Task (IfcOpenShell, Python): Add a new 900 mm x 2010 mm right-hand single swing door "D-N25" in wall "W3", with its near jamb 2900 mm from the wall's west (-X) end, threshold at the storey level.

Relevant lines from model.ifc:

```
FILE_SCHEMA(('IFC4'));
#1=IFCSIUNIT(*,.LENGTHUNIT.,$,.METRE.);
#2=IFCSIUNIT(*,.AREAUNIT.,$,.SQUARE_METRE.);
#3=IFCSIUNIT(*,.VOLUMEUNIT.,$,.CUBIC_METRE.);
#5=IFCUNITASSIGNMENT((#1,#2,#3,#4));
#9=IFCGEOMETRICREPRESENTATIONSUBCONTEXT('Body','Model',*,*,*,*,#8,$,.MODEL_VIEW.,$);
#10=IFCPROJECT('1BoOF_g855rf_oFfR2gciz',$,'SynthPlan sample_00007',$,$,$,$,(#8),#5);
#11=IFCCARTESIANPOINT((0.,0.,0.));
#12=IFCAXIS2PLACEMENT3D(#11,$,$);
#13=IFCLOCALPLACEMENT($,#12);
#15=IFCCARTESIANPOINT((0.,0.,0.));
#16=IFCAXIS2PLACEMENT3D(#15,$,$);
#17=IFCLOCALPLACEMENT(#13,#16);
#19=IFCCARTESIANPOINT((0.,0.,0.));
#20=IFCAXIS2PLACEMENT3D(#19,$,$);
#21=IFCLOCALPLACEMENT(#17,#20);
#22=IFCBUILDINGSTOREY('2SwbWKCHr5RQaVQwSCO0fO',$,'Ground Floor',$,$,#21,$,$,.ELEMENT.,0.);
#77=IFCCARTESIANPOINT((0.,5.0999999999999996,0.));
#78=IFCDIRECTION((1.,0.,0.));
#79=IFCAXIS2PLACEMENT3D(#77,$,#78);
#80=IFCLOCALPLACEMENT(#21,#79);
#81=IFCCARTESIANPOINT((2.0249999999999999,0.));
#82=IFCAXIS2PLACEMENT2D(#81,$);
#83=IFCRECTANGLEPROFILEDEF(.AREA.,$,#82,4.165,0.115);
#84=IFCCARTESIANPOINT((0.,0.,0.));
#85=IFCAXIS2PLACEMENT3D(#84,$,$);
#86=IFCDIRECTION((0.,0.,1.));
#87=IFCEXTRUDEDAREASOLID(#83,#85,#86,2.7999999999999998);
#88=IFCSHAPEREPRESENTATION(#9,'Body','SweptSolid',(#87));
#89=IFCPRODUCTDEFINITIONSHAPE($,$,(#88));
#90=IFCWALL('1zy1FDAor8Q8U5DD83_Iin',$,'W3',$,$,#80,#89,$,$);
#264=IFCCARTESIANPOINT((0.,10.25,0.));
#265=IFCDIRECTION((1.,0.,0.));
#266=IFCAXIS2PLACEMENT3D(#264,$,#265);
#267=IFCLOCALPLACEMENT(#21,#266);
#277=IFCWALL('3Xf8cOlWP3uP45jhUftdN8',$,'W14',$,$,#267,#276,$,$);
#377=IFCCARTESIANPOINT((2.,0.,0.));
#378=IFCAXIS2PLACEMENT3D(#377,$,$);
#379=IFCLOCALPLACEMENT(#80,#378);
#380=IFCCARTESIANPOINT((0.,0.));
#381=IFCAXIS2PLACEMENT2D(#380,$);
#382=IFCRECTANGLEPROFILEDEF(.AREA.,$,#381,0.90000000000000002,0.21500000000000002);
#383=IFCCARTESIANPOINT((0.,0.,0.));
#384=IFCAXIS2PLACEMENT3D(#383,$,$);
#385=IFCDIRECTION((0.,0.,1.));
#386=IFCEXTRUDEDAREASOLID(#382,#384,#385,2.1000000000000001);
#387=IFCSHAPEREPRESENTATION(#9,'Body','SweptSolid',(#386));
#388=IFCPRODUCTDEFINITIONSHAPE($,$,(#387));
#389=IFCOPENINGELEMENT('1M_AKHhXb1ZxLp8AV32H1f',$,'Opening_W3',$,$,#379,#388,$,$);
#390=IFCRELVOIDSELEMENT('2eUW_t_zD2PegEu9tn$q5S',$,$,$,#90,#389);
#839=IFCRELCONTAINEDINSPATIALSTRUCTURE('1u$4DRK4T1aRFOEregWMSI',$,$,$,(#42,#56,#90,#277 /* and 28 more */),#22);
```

```python
import numpy as np
import ifcopenshell
import ifcopenshell.api.feature
import ifcopenshell.api.geometry
import ifcopenshell.api.root
import ifcopenshell.api.spatial
import ifcopenshell.geom
import ifcopenshell.util.element
import ifcopenshell.util.placement
import ifcopenshell.util.representation
import ifcopenshell.util.shape
import ifcopenshell.util.unit

model = ifcopenshell.open("model.ifc")
unit_scale = ifcopenshell.util.unit.calculate_unit_scale(model)
settings = ifcopenshell.geom.settings()


def volume(element):
    """Net volume in cubic metres, openings subtracted."""
    shape = ifcopenshell.geom.create_shape(settings, element)
    return ifcopenshell.util.shape.get_volume(shape.geometry)


wall = model.by_guid("1zy1FDAor8Q8U5DD83_Iin")
storey = ifcopenshell.util.element.get_container(wall, ifc_class="IfcBuildingStorey")
context = ifcopenshell.util.representation.get_context(model, "Model", "Body", "MODEL_VIEW")
before = volume(wall)

width, height, from_end, sill = 0.9, 2.01, 2.9, 0.0  # metres

# The wall runs along its own X axis, and the end named is its -X end.
wall_shape = ifcopenshell.geom.create_shape(settings, wall)
x, y, z = ifcopenshell.util.shape.get_vertices(wall_shape.geometry).T
start = x.min() + from_end
face, thickness = float(y.min()), float(y.max() - y.min())
wall_matrix = ifcopenshell.util.placement.get_local_placement(wall.ObjectPlacement)
level = ifcopenshell.util.placement.get_local_placement(storey.ObjectPlacement)[2, 3]


def in_wall(x, y):
    """Placement at x, y metres in the wall's axes, at sill height."""
    matrix = wall_matrix.copy()
    matrix[:, 3] = wall_matrix @ np.array([x / unit_scale, y / unit_scale, 0.0, 1.0])
    matrix[2, 3] = level + sill / unit_scale
    return matrix


# Opening: a box that overshoots both wall faces by 50 mm.
opening = ifcopenshell.api.root.create_entity(model, ifc_class="IfcOpeningElement", predefined_type="OPENING")
box = ifcopenshell.api.geometry.add_wall_representation(
    model, context=context, length=width, height=height, thickness=thickness + 0.1
)
ifcopenshell.api.geometry.assign_representation(model, product=opening, representation=box)
ifcopenshell.api.geometry.edit_object_placement(model, product=opening, matrix=in_wall(start, face - 0.05), is_si=False)
ifcopenshell.api.feature.add_feature(model, feature=opening, element=wall)

door = ifcopenshell.api.root.create_entity(model, ifc_class="IfcDoor", name="D-N25", predefined_type="DOOR")
door.OverallWidth, door.OverallHeight = width / unit_scale, height / unit_scale
door.OperationType = "SINGLE_SWING_RIGHT"
body = ifcopenshell.api.geometry.add_door_representation(
    model,
    context=context,
    overall_width=door.OverallWidth,
    overall_height=door.OverallHeight,
    operation_type="SINGLE_SWING_RIGHT",
    lining_properties={"LiningDepth": thickness / unit_scale, "ThresholdDepth": thickness / unit_scale},
)
ifcopenshell.api.geometry.assign_representation(model, product=door, representation=body)
ifcopenshell.api.spatial.assign_container(model, products=[door], relating_structure=storey)
ifcopenshell.api.feature.add_filling(model, opening=opening, element=door)

# The lining spans the wall, so the door starts at the wall face.
ifcopenshell.api.geometry.edit_object_placement(model, product=door, matrix=in_wall(start, face), is_si=False)

after = volume(wall)

print(f"wall volume {before:.3f} -> {after:.3f} m3")

model.write("model-out.ifc")
```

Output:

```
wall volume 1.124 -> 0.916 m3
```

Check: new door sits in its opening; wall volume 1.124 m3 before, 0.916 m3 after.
